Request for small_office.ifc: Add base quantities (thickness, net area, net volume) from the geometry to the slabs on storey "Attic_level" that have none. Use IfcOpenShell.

First a look at what the model holds.

```python
import ifcopenshell
import ifcopenshell.util.element
import ifcopenshell.util.unit

model = ifcopenshell.open("small_office.ifc")
print(model.schema)
for unit_type in ("LENGTHUNIT", "AREAUNIT", "VOLUMEUNIT"):
    print(unit_type, ifcopenshell.util.unit.calculate_unit_scale(model, unit_type))
storey = next(s for s in model.by_type("IfcBuildingStorey") if s.Name == "Attic_level")
slabs = [e for e in ifcopenshell.util.element.get_decomposition(storey) if e.is_a("IfcSlab")]
for e in sorted(slabs, key=lambda e: e.id()):
    print(e.id(), e.is_a(), e.Name, list(ifcopenshell.util.element.get_psets(e, qtos_only=True)), sep=" | ")
```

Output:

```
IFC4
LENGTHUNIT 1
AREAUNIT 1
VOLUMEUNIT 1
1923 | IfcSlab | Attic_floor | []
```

```python
import ifcopenshell
import ifcopenshell.api.pset
import ifcopenshell.geom
import ifcopenshell.util.element
import ifcopenshell.util.shape
import ifcopenshell.util.unit

model = ifcopenshell.open("small_office.ifc")
unit_scale = ifcopenshell.util.unit.calculate_unit_scale(model)
area_scale = ifcopenshell.util.unit.calculate_unit_scale(model, "AREAUNIT")
volume_scale = ifcopenshell.util.unit.calculate_unit_scale(model, "VOLUMEUNIT")
settings = ifcopenshell.geom.settings()

storey = next(s for s in model.by_type("IfcBuildingStorey") if s.Name == "Attic_level")
slabs = [e for e in ifcopenshell.util.element.get_decomposition(storey) if e.is_a("IfcSlab")]

for e in sorted(slabs, key=lambda e: e.id()):
    if ifcopenshell.util.element.get_psets(e, qtos_only=True, should_inherit=False):
        continue
    # Geometry comes back in metres, in the element's own axes.
    shape = ifcopenshell.geom.create_shape(settings, e)
    values = {
        "Width": ifcopenshell.util.shape.get_z(shape.geometry) / unit_scale,
        "NetArea": ifcopenshell.util.shape.get_footprint_area(shape.geometry) / area_scale,
        "NetVolume": ifcopenshell.util.shape.get_volume(shape.geometry) / volume_scale,
    }
    qto = ifcopenshell.api.pset.add_qto(model, product=e, name="Qto_SlabBaseQuantities")
    ifcopenshell.api.pset.edit_qto(model, qto=qto, properties=values)
    print(e.id(), {k: round(v, 3) for k, v in values.items()})

model.write("small_office_rev.ifc")
```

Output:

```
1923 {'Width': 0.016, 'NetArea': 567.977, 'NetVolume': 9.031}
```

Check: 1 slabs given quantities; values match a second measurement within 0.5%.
